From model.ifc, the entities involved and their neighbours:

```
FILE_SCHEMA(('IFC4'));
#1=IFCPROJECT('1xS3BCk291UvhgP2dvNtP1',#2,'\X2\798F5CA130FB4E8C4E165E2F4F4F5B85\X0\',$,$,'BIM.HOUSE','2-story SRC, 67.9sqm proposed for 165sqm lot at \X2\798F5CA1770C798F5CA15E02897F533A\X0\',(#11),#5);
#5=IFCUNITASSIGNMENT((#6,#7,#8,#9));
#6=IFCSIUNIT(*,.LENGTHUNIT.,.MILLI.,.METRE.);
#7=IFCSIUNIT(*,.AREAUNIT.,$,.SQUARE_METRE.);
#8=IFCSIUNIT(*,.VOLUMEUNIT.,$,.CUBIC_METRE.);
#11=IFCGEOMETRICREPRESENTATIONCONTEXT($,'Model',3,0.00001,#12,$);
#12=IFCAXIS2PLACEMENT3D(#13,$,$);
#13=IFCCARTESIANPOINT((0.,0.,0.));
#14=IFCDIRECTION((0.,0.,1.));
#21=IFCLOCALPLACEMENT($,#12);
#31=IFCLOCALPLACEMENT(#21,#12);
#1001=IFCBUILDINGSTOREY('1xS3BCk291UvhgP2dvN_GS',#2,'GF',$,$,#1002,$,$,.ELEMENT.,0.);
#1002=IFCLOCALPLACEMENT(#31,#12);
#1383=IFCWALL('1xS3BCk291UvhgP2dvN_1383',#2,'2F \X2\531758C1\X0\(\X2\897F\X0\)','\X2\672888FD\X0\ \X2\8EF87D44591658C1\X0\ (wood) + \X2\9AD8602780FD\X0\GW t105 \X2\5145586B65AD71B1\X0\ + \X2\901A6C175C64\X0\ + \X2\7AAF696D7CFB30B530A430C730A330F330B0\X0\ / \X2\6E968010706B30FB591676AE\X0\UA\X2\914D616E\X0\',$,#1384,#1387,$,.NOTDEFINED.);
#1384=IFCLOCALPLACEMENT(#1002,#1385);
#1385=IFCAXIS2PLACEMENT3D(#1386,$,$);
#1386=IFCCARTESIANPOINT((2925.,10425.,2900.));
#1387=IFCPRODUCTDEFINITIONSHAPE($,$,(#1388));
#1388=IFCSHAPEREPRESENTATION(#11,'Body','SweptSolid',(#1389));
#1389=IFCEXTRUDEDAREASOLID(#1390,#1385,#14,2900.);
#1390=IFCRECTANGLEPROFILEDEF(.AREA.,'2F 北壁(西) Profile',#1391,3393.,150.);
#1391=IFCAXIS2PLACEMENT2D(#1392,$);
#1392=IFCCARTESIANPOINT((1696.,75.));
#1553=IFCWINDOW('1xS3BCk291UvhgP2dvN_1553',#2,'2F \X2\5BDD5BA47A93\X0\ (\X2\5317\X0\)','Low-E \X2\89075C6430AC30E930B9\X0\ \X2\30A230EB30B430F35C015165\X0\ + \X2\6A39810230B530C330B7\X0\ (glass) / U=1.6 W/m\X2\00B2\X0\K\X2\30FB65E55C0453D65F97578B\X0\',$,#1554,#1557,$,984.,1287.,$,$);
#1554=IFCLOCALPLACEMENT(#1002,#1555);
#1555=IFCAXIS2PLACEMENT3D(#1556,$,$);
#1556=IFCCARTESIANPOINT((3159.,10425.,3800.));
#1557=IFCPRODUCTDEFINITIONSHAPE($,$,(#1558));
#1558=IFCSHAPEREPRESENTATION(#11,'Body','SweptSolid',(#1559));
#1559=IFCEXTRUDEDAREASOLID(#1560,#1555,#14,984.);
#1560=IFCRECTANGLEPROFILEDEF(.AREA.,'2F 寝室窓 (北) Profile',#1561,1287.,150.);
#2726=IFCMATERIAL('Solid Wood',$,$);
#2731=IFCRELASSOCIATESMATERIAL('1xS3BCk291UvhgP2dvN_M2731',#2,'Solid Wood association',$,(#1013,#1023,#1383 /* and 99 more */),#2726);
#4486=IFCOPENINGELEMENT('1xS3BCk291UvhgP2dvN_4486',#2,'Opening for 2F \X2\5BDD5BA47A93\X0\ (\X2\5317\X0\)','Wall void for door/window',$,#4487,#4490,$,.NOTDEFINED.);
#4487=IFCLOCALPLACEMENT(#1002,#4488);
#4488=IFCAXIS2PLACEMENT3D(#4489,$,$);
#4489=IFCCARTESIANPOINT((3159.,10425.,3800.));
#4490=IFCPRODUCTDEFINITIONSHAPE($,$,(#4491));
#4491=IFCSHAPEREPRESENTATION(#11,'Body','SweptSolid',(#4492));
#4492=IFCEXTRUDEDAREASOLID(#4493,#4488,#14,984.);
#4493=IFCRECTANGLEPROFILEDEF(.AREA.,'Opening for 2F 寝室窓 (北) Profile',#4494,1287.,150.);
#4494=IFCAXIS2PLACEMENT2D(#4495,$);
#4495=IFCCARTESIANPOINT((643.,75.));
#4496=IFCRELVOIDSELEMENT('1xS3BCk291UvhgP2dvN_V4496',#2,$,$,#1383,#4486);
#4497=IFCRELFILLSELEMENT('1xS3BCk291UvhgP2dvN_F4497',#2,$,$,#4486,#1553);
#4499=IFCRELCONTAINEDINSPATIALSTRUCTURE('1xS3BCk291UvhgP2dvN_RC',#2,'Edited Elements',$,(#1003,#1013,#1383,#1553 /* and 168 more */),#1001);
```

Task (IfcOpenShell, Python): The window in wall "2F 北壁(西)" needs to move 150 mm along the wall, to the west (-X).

```python
import ifcopenshell
import ifcopenshell.api.geometry
import ifcopenshell.util.placement
import ifcopenshell.util.unit

model = ifcopenshell.open("model.ifc")
unit_scale = ifcopenshell.util.unit.calculate_unit_scale(model)

window = model.by_guid("1xS3BCk291UvhgP2dvN_1553")
opening = window.FillsVoids[0].RelatingOpeningElement
wall = opening.VoidsElements[0].RelatingBuildingElement

wall_matrix = ifcopenshell.util.placement.get_local_placement(wall.ObjectPlacement)
shift = wall_matrix[:3, 0] * -0.15 / unit_scale
before = ifcopenshell.util.placement.get_local_placement(window.ObjectPlacement)[:3, 3].copy()

# The window is not placed relative to its opening, so move both.
for product in (opening, window):
    matrix = ifcopenshell.util.placement.get_local_placement(product.ObjectPlacement)
    matrix[:3, 3] += shift
    ifcopenshell.api.geometry.edit_object_placement(model, product=product, matrix=matrix, is_si=False)

after = ifcopenshell.util.placement.get_local_placement(window.ObjectPlacement)[:3, 3]
print("window moved by", (after - before).round(3) + 0.0)

model.write("model_updated.ifc")
```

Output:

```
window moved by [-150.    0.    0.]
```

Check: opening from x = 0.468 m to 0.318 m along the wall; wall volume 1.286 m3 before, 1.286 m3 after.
